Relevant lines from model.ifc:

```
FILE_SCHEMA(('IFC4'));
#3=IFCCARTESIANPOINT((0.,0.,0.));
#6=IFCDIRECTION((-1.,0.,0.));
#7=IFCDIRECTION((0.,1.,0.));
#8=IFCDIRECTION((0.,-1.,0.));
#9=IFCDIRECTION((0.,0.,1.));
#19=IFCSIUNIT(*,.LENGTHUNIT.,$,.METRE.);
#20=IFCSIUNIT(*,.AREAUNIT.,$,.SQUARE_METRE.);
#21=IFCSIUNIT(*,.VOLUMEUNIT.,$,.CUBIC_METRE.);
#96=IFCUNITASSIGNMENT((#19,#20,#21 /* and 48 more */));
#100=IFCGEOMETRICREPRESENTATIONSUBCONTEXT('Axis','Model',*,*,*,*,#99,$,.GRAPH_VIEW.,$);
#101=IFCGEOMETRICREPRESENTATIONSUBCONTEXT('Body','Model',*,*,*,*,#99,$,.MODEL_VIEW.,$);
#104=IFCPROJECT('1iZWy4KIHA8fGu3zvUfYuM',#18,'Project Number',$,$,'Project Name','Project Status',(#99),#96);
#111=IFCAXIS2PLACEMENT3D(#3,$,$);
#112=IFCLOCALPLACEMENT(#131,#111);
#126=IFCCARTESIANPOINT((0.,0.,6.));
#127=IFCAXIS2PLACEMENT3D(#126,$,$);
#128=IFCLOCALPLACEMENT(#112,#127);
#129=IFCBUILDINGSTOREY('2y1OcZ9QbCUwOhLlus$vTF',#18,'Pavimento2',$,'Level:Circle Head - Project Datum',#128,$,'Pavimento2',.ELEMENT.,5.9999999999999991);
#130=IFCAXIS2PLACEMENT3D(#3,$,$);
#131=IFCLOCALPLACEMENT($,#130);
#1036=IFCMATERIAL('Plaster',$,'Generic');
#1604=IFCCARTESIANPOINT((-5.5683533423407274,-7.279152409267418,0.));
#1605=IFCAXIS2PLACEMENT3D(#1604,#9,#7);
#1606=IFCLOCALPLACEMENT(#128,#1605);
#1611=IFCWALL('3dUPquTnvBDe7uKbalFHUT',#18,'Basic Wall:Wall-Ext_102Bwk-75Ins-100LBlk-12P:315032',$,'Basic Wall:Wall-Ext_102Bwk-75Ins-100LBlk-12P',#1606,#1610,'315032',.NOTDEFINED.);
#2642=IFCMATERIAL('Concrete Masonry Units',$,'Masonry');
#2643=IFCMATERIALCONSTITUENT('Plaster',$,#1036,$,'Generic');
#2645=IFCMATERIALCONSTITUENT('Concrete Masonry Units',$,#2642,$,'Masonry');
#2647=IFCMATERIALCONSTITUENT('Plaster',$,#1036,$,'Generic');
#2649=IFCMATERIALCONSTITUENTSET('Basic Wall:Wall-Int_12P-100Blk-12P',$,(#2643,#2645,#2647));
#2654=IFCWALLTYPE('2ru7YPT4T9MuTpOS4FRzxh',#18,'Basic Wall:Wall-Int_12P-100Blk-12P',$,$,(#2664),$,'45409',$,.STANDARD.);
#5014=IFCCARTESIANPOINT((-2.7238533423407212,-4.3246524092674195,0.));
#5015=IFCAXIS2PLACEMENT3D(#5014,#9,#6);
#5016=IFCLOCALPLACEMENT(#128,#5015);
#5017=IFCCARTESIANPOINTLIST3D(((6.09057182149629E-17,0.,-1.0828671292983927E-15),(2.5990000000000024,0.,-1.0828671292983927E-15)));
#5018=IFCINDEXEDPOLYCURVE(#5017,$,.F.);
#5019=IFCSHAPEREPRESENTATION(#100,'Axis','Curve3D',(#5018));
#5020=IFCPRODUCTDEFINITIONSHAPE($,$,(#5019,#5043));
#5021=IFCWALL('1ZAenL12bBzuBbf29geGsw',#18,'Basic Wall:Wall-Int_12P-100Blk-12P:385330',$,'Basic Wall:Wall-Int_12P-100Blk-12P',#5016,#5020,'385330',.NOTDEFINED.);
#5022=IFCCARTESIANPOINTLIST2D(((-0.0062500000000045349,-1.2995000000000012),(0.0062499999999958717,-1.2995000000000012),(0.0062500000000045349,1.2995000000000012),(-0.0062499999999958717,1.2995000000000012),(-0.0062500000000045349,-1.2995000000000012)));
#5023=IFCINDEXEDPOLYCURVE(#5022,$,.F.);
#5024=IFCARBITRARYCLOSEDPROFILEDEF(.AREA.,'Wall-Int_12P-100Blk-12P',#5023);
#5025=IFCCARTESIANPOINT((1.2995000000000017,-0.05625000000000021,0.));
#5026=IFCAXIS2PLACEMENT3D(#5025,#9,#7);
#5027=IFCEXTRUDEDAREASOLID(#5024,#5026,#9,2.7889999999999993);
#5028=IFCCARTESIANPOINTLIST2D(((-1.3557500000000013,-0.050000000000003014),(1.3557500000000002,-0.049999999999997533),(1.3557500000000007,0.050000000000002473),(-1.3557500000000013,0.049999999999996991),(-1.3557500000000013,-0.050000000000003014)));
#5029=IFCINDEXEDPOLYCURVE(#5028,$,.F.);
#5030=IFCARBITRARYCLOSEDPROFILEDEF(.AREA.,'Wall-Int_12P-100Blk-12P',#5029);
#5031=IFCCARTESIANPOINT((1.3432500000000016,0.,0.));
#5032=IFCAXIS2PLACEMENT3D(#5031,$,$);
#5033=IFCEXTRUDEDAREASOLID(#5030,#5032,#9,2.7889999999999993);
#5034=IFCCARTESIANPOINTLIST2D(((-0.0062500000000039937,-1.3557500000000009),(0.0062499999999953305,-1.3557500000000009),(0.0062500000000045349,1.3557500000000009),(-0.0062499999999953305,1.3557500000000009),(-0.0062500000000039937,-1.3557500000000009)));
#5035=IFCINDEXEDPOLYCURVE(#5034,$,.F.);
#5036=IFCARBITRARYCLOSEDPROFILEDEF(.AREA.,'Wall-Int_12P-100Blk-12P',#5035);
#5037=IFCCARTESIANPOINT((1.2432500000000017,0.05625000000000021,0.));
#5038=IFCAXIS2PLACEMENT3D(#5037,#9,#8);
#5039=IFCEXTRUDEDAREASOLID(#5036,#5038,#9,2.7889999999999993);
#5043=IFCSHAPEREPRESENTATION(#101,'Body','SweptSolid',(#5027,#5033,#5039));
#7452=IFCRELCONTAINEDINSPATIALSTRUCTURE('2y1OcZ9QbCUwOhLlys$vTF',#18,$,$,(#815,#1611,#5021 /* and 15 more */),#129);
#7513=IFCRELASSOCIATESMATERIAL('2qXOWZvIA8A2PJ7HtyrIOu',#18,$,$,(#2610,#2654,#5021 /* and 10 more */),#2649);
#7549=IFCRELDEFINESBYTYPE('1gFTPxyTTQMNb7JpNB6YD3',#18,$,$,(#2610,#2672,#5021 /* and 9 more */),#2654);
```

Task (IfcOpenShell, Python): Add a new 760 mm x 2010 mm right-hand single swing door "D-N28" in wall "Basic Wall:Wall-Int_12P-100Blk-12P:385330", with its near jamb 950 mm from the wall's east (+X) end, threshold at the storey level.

```python
import numpy as np
import ifcopenshell
import ifcopenshell.api.feature
import ifcopenshell.api.geometry
import ifcopenshell.api.root
import ifcopenshell.api.spatial
import ifcopenshell.geom
import ifcopenshell.util.element
import ifcopenshell.util.placement
import ifcopenshell.util.representation
import ifcopenshell.util.shape
import ifcopenshell.util.unit

model = ifcopenshell.open("model.ifc")
unit_scale = ifcopenshell.util.unit.calculate_unit_scale(model)
settings = ifcopenshell.geom.settings()


def volume(element):
    """Net volume in cubic metres, openings subtracted."""
    shape = ifcopenshell.geom.create_shape(settings, element)
    return ifcopenshell.util.shape.get_volume(shape.geometry)


wall = model.by_guid("1ZAenL12bBzuBbf29geGsw")
storey = ifcopenshell.util.element.get_container(wall, ifc_class="IfcBuildingStorey")
context = ifcopenshell.util.representation.get_context(model, "Model", "Body", "MODEL_VIEW")
before = volume(wall)

width, height, from_end, sill = 0.76, 2.01, 0.95, 0.0  # metres

# The wall runs along its own X axis, and the end named is its -X end.
wall_shape = ifcopenshell.geom.create_shape(settings, wall)
x, y, z = ifcopenshell.util.shape.get_vertices(wall_shape.geometry).T
start = x.min() + from_end
face, thickness = float(y.min()), float(y.max() - y.min())
wall_matrix = ifcopenshell.util.placement.get_local_placement(wall.ObjectPlacement)
level = ifcopenshell.util.placement.get_local_placement(storey.ObjectPlacement)[2, 3]


def in_wall(x, y):
    """Placement at x, y metres in the wall's axes, at sill height."""
    matrix = wall_matrix.copy()
    matrix[:, 3] = wall_matrix @ np.array([x / unit_scale, y / unit_scale, 0.0, 1.0])
    matrix[2, 3] = level + sill / unit_scale
    return matrix


# Opening: a box that overshoots both wall faces by 50 mm.
opening = ifcopenshell.api.root.create_entity(model, ifc_class="IfcOpeningElement", predefined_type="OPENING")
box = ifcopenshell.api.geometry.add_wall_representation(
    model, context=context, length=width, height=height, thickness=thickness + 0.1
)
ifcopenshell.api.geometry.assign_representation(model, product=opening, representation=box)
ifcopenshell.api.geometry.edit_object_placement(model, product=opening, matrix=in_wall(start, face - 0.05), is_si=False)
ifcopenshell.api.feature.add_feature(model, feature=opening, element=wall)

door = ifcopenshell.api.root.create_entity(model, ifc_class="IfcDoor", name="D-N28", predefined_type="DOOR")
door.OverallWidth, door.OverallHeight = width / unit_scale, height / unit_scale
door.OperationType = "SINGLE_SWING_RIGHT"
body = ifcopenshell.api.geometry.add_door_representation(
    model,
    context=context,
    overall_width=door.OverallWidth,
    overall_height=door.OverallHeight,
    operation_type="SINGLE_SWING_RIGHT",
    lining_properties={"LiningDepth": thickness / unit_scale, "ThresholdDepth": thickness / unit_scale},
)
ifcopenshell.api.geometry.assign_representation(model, product=door, representation=body)
ifcopenshell.api.spatial.assign_container(model, products=[door], relating_structure=storey)
ifcopenshell.api.feature.add_filling(model, opening=opening, element=door)

# The lining spans the wall, so the door starts at the wall face.
ifcopenshell.api.geometry.edit_object_placement(model, product=door, matrix=in_wall(start, face), is_si=False)

after = volume(wall)

print(f"wall volume {before:.3f} -> {after:.3f} m3")

model.write("model_rev.ifc")
```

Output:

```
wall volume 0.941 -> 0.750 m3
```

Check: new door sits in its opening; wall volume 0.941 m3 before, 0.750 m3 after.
